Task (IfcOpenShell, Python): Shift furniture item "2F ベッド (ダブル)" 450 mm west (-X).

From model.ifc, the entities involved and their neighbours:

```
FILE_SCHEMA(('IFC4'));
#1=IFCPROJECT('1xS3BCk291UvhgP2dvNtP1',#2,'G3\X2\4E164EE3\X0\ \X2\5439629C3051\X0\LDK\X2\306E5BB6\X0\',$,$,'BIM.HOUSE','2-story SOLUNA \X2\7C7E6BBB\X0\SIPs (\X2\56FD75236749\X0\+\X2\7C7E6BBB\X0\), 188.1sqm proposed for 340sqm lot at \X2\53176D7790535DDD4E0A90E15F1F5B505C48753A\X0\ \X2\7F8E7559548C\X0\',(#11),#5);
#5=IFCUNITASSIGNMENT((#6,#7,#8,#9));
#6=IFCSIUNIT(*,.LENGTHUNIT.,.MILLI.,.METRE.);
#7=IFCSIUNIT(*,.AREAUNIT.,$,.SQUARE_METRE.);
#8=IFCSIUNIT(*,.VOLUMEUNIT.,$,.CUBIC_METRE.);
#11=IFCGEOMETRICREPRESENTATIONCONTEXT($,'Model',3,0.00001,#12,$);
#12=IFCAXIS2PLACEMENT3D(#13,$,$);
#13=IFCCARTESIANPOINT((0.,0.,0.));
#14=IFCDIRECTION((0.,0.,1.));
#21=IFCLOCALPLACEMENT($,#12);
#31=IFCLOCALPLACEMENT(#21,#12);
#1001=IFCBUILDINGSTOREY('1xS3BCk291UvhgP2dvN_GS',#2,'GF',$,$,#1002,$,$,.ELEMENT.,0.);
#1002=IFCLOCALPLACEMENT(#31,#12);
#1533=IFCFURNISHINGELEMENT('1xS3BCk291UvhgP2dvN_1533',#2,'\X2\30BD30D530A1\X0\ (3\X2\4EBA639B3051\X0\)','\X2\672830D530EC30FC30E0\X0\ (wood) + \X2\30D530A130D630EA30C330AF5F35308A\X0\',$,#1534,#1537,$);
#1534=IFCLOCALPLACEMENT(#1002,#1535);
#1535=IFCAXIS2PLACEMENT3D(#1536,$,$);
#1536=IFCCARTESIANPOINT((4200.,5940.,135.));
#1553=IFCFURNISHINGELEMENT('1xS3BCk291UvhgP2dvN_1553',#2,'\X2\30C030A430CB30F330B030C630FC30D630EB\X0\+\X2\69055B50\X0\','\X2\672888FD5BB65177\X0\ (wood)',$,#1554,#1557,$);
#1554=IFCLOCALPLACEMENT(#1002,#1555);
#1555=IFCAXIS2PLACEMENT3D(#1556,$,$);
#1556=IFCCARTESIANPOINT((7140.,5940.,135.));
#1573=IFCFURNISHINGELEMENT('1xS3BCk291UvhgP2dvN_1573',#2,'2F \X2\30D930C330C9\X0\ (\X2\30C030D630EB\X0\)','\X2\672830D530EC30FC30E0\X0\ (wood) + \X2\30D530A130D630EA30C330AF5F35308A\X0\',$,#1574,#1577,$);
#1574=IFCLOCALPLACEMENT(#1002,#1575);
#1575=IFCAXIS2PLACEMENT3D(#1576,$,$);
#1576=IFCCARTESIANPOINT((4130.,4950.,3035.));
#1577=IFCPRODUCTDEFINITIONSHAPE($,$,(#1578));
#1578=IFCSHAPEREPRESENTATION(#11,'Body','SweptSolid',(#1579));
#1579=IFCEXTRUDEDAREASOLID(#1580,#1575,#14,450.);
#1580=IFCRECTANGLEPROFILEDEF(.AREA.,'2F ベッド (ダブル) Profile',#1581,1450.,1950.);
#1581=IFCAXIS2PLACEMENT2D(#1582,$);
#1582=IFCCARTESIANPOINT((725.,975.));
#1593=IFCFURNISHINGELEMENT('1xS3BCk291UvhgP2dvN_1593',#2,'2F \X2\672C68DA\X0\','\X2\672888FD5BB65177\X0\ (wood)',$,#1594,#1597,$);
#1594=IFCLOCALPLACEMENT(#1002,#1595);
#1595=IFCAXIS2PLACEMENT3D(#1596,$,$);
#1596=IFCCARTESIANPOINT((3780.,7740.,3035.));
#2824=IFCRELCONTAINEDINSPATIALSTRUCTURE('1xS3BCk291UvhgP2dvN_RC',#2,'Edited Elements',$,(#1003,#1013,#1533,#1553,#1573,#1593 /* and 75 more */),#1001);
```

```python
import ifcopenshell
import ifcopenshell.api.geometry
import ifcopenshell.util.placement
import ifcopenshell.util.unit

model = ifcopenshell.open("model.ifc")
unit_scale = ifcopenshell.util.unit.calculate_unit_scale(model)

item = model.by_guid("1xS3BCk291UvhgP2dvN_1573")
matrix = ifcopenshell.util.placement.get_local_placement(item.ObjectPlacement)
matrix[0, 3] -= 0.45 / unit_scale
ifcopenshell.api.geometry.edit_object_placement(model, product=item, matrix=matrix, is_si=False)

print(ifcopenshell.util.placement.get_local_placement(item.ObjectPlacement).round(3) + 0.0)

model.write("model_v2.ifc")
```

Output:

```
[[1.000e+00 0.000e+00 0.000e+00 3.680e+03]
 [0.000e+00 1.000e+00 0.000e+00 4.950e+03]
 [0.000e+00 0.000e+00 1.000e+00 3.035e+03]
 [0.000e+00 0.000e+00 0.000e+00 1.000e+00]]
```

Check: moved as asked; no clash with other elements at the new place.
